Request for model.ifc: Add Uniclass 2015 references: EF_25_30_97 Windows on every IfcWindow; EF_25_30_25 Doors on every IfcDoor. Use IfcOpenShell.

First a look at what the model holds.

```python
import ifcopenshell

model = ifcopenshell.open("model.ifc")
print(model.schema)
print("classifications:", [c.Name for c in model.by_type("IfcClassification")])
for ifc_class in ("IfcDoor", "IfcRoof", "IfcStair", "IfcWall", "IfcWindow"):
    print(ifc_class, len(model.by_type(ifc_class)))
```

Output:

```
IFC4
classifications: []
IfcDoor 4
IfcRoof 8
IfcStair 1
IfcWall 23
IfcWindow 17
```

```python
import ifcopenshell
import ifcopenshell.api.classification

model = ifcopenshell.open("model.ifc")

system = ifcopenshell.api.classification.add_classification(model, classification="Uniclass 2015")

codes = {
    "IfcWindow": ("EF_25_30_97", "Windows"),
    "IfcDoor": ("EF_25_30_25", "Doors"),
}
for ifc_class, (code, name) in codes.items():
    products = model.by_type(ifc_class)
    ifcopenshell.api.classification.add_reference(
        model, products=products, classification=system, identification=code, name=name
    )
    print(code, len(products))

model.write("model_rev.ifc")
```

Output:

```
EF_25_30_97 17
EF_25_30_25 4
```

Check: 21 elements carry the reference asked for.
